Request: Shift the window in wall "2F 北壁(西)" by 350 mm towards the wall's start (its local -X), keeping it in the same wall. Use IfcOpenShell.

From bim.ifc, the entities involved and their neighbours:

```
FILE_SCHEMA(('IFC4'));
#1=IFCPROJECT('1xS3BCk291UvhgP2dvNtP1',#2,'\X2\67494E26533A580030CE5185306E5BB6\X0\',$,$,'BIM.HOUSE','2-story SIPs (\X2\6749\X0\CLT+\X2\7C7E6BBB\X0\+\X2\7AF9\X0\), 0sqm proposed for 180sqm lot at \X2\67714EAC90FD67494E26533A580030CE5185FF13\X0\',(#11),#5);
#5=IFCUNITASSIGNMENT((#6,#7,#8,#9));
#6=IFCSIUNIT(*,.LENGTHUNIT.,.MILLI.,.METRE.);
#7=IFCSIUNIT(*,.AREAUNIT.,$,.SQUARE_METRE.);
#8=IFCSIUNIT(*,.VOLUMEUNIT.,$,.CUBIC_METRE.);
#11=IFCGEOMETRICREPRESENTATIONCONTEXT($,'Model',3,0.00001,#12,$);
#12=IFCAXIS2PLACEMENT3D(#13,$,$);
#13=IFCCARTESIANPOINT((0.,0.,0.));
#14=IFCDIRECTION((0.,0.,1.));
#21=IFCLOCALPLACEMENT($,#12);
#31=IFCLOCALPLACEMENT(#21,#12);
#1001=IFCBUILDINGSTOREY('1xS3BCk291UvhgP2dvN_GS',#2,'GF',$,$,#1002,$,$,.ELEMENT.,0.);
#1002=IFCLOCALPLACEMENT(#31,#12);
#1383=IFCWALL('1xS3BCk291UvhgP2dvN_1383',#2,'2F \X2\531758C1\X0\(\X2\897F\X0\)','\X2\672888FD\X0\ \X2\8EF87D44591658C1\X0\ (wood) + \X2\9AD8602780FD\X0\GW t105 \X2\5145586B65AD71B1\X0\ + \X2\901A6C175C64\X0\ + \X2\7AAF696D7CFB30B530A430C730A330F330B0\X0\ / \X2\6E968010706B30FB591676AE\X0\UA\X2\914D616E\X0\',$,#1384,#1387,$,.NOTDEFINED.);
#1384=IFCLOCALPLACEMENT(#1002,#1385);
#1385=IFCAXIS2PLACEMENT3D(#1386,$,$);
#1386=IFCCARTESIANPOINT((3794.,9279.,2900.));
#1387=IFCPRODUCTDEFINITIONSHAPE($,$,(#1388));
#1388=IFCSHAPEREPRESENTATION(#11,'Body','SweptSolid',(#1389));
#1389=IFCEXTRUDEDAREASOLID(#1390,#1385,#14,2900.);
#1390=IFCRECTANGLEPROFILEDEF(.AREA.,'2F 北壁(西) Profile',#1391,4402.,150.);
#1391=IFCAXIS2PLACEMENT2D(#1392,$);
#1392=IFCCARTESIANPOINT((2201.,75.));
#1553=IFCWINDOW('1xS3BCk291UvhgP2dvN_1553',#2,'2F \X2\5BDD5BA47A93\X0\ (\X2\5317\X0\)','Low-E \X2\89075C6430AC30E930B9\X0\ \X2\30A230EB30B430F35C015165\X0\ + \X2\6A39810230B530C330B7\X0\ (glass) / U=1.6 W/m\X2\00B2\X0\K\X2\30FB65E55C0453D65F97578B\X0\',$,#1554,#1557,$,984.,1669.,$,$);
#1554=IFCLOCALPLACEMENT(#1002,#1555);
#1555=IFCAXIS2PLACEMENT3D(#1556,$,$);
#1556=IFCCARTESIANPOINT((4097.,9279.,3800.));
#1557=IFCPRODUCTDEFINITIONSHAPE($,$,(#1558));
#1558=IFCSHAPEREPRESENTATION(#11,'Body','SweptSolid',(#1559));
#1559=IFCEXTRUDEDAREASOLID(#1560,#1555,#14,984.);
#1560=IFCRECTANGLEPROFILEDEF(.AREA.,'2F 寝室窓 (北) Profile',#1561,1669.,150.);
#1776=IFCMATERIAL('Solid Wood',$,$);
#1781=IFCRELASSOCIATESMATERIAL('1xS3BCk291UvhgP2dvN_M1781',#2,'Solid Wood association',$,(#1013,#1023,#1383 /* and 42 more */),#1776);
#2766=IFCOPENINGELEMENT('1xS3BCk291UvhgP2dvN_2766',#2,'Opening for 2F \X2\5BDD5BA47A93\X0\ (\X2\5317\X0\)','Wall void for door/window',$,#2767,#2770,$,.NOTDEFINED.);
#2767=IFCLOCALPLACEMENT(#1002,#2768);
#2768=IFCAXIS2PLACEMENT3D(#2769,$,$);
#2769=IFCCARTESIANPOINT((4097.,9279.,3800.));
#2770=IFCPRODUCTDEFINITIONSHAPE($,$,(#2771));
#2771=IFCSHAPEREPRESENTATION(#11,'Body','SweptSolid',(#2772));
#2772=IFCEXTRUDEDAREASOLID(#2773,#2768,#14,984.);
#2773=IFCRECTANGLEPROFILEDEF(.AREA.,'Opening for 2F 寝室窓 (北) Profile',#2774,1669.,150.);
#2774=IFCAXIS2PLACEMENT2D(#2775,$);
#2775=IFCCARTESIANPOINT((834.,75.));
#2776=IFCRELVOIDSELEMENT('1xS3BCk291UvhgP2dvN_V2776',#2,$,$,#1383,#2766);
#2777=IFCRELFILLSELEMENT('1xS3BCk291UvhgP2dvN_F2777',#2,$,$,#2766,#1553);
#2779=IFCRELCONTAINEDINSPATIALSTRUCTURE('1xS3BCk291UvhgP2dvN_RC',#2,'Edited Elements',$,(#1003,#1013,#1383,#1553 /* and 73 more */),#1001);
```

```python
import ifcopenshell
import ifcopenshell.api.geometry
import ifcopenshell.util.placement

model = ifcopenshell.open("bim.ifc")

window = model.by_guid("1xS3BCk291UvhgP2dvN_1553")
opening = window.FillsVoids[0].RelatingOpeningElement
wall = opening.VoidsElements[0].RelatingBuildingElement

wall_matrix = ifcopenshell.util.placement.get_local_placement(wall.ObjectPlacement)
shift = wall_matrix[:3, 0] * -350.0
before = ifcopenshell.util.placement.get_local_placement(window.ObjectPlacement)[:3, 3].copy()

# The window is not placed relative to its opening, so move both.
for product in (opening, window):
    matrix = ifcopenshell.util.placement.get_local_placement(product.ObjectPlacement)
    matrix[:3, 3] += shift
    ifcopenshell.api.geometry.edit_object_placement(model, product=product, matrix=matrix, is_si=False)

after = ifcopenshell.util.placement.get_local_placement(window.ObjectPlacement)[:3, 3]
print("window moved by", (after - before).round(3) + 0.0)

model.write("bim-out.ifc")
```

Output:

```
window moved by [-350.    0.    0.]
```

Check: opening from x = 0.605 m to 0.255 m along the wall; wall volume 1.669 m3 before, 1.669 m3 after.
